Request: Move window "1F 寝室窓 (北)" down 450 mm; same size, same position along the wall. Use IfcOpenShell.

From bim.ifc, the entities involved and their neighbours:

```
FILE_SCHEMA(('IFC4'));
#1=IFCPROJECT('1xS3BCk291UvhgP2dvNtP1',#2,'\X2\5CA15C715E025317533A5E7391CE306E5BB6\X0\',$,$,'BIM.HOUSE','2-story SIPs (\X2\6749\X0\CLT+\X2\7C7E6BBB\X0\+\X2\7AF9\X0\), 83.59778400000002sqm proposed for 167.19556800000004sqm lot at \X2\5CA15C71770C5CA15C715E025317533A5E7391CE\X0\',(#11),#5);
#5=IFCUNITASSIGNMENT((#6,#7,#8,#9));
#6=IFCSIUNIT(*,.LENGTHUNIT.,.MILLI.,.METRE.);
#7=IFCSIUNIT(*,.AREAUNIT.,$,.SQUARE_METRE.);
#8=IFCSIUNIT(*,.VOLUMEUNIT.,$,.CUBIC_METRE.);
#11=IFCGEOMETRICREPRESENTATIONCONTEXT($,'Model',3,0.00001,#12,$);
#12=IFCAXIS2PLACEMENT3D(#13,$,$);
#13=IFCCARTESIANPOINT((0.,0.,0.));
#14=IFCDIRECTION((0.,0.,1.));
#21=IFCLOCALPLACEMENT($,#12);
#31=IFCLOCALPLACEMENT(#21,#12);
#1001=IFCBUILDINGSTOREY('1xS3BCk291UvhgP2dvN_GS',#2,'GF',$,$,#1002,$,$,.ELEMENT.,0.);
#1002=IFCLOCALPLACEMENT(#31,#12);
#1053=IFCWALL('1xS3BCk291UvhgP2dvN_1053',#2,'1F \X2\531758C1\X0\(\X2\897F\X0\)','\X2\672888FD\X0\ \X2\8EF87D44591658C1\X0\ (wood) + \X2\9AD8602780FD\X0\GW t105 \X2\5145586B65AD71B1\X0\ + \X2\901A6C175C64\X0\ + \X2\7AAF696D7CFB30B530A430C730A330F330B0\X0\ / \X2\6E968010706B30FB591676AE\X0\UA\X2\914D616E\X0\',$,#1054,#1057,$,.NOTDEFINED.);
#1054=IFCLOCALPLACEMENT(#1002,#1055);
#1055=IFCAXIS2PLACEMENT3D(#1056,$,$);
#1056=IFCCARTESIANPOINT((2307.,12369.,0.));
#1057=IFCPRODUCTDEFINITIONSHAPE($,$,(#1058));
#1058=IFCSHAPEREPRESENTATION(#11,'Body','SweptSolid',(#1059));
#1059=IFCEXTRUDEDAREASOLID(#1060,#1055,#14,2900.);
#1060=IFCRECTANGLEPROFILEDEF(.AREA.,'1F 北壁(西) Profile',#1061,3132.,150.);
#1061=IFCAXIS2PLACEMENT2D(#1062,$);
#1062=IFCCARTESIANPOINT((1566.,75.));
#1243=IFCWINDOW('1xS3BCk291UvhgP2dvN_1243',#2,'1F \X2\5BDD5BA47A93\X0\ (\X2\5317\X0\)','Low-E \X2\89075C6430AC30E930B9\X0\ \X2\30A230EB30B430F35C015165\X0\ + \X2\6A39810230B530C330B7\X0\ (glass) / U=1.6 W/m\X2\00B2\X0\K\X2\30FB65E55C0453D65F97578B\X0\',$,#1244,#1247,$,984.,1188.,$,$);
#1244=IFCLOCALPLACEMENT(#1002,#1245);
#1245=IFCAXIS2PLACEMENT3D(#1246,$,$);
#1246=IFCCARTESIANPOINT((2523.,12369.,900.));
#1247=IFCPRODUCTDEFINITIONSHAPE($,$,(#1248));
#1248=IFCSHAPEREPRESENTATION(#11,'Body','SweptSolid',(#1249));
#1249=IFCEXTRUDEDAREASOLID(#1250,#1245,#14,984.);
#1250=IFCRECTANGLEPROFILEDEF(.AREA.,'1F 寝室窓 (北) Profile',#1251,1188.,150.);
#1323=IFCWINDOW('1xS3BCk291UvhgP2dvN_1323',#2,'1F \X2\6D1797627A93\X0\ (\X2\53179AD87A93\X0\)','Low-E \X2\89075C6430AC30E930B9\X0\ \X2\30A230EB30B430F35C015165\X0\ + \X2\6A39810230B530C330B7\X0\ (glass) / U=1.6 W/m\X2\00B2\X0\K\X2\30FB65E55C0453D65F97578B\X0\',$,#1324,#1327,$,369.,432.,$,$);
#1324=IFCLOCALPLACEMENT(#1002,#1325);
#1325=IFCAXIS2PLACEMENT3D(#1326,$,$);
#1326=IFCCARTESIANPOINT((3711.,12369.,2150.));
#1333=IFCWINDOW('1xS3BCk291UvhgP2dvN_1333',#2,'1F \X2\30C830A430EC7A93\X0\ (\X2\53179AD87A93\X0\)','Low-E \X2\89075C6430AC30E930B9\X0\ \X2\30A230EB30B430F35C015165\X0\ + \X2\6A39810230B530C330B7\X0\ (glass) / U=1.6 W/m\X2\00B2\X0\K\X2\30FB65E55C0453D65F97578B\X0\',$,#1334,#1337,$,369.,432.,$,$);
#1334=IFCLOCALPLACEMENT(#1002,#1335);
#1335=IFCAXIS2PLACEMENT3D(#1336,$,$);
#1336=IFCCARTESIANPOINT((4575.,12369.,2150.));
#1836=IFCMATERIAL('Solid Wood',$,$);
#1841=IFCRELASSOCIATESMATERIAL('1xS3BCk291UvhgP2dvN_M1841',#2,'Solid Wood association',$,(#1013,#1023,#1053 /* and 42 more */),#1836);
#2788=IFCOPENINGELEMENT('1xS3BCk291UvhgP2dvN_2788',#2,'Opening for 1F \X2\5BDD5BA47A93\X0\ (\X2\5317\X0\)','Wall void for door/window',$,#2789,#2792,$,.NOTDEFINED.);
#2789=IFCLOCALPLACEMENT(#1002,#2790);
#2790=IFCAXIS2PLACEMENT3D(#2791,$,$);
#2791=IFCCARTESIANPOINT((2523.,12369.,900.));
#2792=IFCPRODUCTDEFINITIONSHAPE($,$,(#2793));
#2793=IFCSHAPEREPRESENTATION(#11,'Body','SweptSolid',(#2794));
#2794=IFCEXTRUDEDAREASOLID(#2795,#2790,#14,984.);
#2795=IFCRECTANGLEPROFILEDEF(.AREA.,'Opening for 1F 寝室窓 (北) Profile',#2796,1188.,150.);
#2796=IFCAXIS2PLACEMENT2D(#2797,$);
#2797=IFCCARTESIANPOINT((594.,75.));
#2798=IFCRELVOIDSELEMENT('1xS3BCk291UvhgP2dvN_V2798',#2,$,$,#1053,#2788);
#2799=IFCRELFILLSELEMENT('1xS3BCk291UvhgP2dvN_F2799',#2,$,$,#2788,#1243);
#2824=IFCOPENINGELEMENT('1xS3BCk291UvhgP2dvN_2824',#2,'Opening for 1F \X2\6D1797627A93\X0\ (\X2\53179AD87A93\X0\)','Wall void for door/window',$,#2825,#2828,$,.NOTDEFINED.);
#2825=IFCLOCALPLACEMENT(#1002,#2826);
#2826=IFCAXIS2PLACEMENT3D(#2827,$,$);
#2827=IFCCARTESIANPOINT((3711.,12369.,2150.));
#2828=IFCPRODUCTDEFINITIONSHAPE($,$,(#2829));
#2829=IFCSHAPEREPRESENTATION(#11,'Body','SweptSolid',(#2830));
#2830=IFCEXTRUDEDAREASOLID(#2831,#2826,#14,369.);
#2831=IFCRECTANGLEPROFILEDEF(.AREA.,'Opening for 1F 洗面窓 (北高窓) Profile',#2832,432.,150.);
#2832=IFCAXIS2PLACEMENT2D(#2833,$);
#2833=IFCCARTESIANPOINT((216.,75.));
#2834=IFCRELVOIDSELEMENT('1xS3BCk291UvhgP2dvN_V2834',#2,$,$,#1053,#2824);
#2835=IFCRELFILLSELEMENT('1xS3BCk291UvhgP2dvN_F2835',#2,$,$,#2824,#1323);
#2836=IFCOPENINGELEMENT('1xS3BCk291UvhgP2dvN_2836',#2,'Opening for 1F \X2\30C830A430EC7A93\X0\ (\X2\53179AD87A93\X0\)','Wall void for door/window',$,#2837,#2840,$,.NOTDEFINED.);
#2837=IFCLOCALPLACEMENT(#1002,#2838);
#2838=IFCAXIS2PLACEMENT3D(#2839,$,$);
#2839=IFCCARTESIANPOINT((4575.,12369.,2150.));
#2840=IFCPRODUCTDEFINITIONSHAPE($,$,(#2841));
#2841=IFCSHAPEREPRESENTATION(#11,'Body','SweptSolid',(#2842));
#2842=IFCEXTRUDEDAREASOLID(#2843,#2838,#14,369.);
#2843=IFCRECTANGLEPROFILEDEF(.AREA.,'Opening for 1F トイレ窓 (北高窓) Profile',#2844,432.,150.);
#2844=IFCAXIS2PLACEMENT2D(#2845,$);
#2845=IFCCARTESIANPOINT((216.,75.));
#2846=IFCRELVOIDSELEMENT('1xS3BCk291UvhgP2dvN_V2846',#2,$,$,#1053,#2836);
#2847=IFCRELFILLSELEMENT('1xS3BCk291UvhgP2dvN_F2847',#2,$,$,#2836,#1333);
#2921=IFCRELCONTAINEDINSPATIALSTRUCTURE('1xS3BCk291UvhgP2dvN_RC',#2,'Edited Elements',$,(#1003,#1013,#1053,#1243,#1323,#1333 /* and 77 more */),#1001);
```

```python
import numpy as np
import ifcopenshell
import ifcopenshell.api.geometry
import ifcopenshell.util.placement
import ifcopenshell.util.unit

model = ifcopenshell.open("bim.ifc")
unit_scale = ifcopenshell.util.unit.calculate_unit_scale(model)

window = model.by_guid("1xS3BCk291UvhgP2dvN_1243")
opening = window.FillsVoids[0].RelatingOpeningElement
dz = -0.45 / unit_scale

shift = np.array([0.0, 0.0, dz])
# The window is not placed relative to its opening, so move both.
for product in (opening, window):
    matrix = ifcopenshell.util.placement.get_local_placement(product.ObjectPlacement)
    matrix[:3, 3] += shift
    ifcopenshell.api.geometry.edit_object_placement(model, product=product, matrix=matrix, is_si=False)

print(f"moved by {dz * unit_scale:+.3f} m")

model.write("bim_updated.ifc")
```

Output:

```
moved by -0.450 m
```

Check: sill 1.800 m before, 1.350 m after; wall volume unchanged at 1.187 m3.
